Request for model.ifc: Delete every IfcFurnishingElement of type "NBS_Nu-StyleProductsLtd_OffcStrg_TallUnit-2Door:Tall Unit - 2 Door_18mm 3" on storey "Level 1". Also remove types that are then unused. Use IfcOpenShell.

First a look at what the model holds.

```python
import ifcopenshell
import ifcopenshell.util.element

model = ifcopenshell.open("model.ifc")
print(model.schema)
storey = next(s for s in model.by_type("IfcBuildingStorey") if s.Name == "Level 1")
furniture = [e for e in ifcopenshell.util.element.get_decomposition(storey) if e.is_a("IfcFurnishingElement")]
seen = {}
for e in furniture:
    element_type = ifcopenshell.util.element.get_type(e)
    name = element_type.Name if element_type not in (None, e) else None
    seen[name] = seen.get(name, 0) + 1
for name, count in sorted(seen.items(), key=str):
    print(count, "x", name)
```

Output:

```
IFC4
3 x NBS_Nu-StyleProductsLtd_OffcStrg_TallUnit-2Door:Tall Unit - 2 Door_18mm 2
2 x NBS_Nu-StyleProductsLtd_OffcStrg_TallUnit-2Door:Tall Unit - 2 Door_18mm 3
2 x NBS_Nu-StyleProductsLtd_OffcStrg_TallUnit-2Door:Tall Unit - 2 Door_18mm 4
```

```python
import ifcopenshell
import ifcopenshell.api.root
import ifcopenshell.util.element

model = ifcopenshell.open("model.ifc")

storey = next(s for s in model.by_type("IfcBuildingStorey") if s.Name == "Level 1")
furniture = [e for e in ifcopenshell.util.element.get_decomposition(storey) if e.is_a("IfcFurnishingElement")]
targets = [e for e in furniture if (t := ifcopenshell.util.element.get_type(e)) not in (None, e) and t.Name == "NBS_Nu-StyleProductsLtd_OffcStrg_TallUnit-2Door:Tall Unit - 2 Door_18mm 3"]
types = {ifcopenshell.util.element.get_type(e) for e in targets} - {None, *targets}

for e in targets:
    ifcopenshell.api.root.remove_product(model, product=e)
print(len(targets), "removed")

unused = [t for t in types if not ifcopenshell.util.element.get_types(t)]
for t in unused:
    ifcopenshell.api.root.remove_product(model, product=t)
print(len(unused), "unused types removed")

model.write("model_rev.ifc")
```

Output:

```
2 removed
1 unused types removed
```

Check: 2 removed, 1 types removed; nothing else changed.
